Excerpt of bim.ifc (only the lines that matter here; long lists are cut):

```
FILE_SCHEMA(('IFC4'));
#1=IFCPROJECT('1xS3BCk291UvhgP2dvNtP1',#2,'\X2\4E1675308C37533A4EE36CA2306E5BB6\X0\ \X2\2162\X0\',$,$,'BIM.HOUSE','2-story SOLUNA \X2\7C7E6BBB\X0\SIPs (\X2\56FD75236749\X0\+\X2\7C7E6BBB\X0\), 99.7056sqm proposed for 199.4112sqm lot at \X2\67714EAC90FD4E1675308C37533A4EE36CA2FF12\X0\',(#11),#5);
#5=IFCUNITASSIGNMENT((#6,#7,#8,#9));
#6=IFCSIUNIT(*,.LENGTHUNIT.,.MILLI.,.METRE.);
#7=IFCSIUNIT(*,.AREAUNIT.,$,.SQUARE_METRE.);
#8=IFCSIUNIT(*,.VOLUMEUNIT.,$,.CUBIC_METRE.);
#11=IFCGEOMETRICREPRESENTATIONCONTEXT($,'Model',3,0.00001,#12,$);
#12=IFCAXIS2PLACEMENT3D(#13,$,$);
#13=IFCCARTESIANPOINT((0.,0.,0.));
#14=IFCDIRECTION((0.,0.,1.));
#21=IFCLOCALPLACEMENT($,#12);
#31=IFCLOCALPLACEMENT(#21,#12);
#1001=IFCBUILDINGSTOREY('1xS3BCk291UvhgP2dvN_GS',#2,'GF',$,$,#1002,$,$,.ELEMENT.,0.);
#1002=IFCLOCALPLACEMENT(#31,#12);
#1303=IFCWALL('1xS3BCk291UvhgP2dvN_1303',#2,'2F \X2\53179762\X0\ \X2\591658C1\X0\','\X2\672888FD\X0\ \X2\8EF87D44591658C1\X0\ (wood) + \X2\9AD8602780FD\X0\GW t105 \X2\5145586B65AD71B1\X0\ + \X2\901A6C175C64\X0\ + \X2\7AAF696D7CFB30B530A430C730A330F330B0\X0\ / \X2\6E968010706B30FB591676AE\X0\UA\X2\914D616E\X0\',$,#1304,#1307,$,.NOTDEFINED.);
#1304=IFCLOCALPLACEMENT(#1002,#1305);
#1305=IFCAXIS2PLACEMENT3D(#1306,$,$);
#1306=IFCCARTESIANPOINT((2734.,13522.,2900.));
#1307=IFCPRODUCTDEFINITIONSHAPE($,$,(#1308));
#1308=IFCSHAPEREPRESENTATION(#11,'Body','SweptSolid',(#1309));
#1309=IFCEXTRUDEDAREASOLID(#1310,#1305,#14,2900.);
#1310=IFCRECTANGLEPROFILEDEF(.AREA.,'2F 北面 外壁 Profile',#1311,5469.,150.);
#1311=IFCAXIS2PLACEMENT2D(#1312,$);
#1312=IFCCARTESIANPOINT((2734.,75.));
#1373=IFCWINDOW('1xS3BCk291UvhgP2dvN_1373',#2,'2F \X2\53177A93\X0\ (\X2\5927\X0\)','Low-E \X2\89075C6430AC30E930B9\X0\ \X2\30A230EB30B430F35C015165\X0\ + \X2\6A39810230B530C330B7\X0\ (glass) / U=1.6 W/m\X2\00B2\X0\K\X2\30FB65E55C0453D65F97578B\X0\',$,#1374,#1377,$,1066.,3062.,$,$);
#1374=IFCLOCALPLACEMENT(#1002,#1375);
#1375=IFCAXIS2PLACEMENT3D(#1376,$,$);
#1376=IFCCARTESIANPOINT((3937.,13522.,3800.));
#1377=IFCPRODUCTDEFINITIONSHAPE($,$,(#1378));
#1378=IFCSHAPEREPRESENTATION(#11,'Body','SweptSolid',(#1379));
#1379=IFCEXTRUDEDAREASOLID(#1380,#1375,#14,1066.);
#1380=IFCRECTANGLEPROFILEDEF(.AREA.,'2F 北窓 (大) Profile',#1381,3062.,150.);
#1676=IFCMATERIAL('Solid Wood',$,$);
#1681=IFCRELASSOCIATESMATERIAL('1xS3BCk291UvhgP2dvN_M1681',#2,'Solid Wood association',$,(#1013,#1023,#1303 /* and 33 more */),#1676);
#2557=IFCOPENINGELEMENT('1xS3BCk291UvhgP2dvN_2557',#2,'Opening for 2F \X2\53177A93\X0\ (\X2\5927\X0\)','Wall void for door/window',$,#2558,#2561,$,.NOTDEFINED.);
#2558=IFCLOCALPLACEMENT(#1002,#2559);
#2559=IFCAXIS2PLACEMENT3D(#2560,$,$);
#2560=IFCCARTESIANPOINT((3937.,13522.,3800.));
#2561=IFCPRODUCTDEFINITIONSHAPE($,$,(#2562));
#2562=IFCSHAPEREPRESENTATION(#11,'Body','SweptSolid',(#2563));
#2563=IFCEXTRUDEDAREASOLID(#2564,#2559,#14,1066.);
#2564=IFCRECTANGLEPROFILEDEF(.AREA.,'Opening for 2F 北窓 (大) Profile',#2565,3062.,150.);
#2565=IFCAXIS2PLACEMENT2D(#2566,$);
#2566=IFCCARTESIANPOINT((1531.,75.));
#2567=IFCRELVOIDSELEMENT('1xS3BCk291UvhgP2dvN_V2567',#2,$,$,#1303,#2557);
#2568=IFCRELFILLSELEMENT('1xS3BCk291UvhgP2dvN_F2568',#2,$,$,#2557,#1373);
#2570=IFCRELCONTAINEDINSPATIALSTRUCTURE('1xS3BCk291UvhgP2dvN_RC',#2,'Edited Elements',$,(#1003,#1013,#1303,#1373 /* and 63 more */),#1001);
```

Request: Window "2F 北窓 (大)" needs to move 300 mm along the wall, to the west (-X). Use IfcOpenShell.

```python
import ifcopenshell
import ifcopenshell.api.geometry
import ifcopenshell.util.placement
import ifcopenshell.util.unit

model = ifcopenshell.open("bim.ifc")
unit_scale = ifcopenshell.util.unit.calculate_unit_scale(model)

window = model.by_guid("1xS3BCk291UvhgP2dvN_1373")
opening = window.FillsVoids[0].RelatingOpeningElement
wall = opening.VoidsElements[0].RelatingBuildingElement

wall_matrix = ifcopenshell.util.placement.get_local_placement(wall.ObjectPlacement)
shift = wall_matrix[:3, 0] * -0.3 / unit_scale
before = ifcopenshell.util.placement.get_local_placement(window.ObjectPlacement)[:3, 3].copy()

# The window is not placed relative to its opening, so move both.
for product in (opening, window):
    matrix = ifcopenshell.util.placement.get_local_placement(product.ObjectPlacement)
    matrix[:3, 3] += shift
    ifcopenshell.api.geometry.edit_object_placement(model, product=product, matrix=matrix, is_si=False)

after = ifcopenshell.util.placement.get_local_placement(window.ObjectPlacement)[:3, 3]
print("window moved by", (after - before).round(3) + 0.0)

model.write("bim-out.ifc")
```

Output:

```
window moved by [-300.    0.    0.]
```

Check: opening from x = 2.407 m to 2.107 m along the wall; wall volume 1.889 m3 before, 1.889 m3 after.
